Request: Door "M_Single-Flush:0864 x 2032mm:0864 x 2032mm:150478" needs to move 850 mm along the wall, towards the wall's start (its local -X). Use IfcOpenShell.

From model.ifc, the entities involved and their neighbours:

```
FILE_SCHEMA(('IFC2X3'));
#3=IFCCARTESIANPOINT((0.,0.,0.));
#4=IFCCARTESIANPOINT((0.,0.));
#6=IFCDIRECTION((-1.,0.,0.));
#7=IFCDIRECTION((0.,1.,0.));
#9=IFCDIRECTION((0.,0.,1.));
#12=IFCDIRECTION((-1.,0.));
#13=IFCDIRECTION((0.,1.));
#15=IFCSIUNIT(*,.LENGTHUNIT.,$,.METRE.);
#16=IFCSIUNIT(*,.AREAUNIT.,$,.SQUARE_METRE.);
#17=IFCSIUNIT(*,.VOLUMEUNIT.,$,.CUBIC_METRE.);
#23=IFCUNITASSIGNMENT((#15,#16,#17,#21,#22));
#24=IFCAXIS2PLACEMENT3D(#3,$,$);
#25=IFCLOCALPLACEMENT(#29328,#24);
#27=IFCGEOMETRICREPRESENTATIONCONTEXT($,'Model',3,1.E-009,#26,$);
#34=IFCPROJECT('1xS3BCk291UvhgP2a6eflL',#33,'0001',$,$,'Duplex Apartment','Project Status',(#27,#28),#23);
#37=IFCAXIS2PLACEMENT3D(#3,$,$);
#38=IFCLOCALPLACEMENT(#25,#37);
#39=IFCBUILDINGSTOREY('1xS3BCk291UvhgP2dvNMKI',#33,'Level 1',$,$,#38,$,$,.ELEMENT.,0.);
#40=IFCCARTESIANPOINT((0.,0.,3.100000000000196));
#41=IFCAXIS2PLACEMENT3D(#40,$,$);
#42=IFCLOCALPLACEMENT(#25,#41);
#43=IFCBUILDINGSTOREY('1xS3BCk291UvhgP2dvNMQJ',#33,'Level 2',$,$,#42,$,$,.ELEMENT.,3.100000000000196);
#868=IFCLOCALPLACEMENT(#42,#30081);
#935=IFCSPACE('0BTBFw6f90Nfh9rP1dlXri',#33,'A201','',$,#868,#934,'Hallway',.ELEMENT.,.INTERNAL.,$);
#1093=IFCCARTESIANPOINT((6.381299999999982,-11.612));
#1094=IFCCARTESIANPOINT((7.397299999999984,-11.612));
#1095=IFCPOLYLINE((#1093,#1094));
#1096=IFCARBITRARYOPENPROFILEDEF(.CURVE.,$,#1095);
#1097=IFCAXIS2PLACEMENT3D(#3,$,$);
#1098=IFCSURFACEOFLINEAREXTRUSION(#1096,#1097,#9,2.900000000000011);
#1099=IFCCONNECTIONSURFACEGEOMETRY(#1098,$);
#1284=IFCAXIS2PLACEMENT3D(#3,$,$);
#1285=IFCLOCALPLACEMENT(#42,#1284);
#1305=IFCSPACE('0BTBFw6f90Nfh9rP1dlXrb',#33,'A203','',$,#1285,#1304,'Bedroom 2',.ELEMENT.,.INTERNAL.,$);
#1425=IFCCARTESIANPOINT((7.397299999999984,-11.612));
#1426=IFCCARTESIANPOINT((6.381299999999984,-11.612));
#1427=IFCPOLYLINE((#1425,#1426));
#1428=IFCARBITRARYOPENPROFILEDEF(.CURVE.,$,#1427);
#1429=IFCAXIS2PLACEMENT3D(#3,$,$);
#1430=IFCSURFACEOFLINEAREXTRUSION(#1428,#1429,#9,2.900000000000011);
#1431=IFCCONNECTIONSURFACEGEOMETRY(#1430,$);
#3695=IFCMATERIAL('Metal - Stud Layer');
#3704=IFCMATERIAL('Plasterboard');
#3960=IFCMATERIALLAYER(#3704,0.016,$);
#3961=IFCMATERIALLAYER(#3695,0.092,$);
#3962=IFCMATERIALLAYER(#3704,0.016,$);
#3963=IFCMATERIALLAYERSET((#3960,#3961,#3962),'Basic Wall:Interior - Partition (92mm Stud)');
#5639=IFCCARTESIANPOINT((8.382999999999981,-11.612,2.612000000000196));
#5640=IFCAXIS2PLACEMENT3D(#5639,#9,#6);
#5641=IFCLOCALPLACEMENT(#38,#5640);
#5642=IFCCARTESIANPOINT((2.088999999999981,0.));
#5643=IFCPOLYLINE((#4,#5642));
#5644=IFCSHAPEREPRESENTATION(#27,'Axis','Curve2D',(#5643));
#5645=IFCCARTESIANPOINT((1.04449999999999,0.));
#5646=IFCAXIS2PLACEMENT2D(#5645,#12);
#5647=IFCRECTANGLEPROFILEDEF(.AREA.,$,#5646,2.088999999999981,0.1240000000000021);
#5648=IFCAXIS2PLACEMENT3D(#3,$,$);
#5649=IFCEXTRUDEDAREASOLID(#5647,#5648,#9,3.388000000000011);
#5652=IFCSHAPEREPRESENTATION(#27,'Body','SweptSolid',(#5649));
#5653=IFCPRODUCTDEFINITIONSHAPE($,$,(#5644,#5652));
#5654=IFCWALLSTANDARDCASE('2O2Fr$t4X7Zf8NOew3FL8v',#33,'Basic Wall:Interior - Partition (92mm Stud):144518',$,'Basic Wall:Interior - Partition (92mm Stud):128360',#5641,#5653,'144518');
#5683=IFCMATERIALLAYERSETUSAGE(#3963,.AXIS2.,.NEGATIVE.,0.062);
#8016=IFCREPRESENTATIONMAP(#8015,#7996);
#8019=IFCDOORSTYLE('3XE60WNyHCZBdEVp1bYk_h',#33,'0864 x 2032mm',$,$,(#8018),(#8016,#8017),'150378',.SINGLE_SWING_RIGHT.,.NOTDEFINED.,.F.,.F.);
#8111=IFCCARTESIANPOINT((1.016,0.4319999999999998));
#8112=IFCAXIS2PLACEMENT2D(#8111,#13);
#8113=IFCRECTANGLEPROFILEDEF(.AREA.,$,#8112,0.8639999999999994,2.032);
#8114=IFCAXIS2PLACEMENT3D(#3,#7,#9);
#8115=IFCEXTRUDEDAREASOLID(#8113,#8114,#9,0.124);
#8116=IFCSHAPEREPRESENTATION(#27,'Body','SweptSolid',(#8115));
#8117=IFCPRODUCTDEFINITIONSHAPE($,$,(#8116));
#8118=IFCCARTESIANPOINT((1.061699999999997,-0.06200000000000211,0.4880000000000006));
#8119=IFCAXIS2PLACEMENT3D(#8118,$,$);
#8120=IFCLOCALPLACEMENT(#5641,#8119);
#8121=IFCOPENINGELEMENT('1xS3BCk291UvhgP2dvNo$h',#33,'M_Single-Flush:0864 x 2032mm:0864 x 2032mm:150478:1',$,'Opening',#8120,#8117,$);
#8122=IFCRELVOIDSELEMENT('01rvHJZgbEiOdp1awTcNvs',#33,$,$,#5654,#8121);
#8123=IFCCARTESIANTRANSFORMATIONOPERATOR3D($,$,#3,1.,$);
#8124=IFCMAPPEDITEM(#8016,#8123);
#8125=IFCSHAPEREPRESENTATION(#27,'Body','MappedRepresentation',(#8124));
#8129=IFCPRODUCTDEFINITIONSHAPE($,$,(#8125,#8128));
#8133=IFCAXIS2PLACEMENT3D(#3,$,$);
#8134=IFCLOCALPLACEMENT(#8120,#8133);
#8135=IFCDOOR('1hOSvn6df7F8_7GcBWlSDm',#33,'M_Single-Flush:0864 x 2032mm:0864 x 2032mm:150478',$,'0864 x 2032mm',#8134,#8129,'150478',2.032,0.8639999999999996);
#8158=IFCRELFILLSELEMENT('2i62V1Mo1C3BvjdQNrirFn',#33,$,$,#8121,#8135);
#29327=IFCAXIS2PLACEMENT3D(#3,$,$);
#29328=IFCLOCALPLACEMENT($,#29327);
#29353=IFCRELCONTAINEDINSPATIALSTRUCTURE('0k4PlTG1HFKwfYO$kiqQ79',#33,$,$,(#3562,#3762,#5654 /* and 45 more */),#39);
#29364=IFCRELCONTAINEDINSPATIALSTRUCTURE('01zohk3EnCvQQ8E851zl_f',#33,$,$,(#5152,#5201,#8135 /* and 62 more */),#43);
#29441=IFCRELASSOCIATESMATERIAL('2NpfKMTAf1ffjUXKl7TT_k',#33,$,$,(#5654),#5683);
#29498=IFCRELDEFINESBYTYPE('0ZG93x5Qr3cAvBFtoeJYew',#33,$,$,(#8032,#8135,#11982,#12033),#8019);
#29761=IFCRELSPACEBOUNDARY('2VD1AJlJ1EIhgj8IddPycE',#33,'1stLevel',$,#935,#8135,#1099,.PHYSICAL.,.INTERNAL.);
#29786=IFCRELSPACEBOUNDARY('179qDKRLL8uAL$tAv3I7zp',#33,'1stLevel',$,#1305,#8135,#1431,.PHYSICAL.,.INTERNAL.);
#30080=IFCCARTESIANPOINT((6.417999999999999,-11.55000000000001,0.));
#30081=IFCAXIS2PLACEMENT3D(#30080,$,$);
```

```python
import numpy as np
import ifcopenshell
import ifcopenshell.api.geometry
import ifcopenshell.util.placement
import ifcopenshell.util.unit

model = ifcopenshell.open("model.ifc")
unit_scale = ifcopenshell.util.unit.calculate_unit_scale(model)

door = model.by_guid("1hOSvn6df7F8_7GcBWlSDm")
opening = door.FillsVoids[0].RelatingOpeningElement
wall = opening.VoidsElements[0].RelatingBuildingElement

wall_matrix = ifcopenshell.util.placement.get_local_placement(wall.ObjectPlacement)
shift = wall_matrix[:3, 0] * -0.85 / unit_scale
before = ifcopenshell.util.placement.get_local_placement(door.ObjectPlacement)[:3, 3].copy()

# The door is placed relative to its opening, so it follows when the opening moves.
matrix = ifcopenshell.util.placement.get_local_placement(opening.ObjectPlacement)
matrix[:3, 3] += shift
ifcopenshell.api.geometry.edit_object_placement(
    model, product=opening, matrix=matrix, is_si=False, should_transform_children=True
)

# Space boundary surfaces are stored in each space's coordinates; move them too.
for rel in door.ProvidesBoundaries:
    if not rel.ConnectionGeometry:
        continue
    surface = rel.ConnectionGeometry.SurfaceOnRelatingElement
    space_matrix = ifcopenshell.util.placement.get_local_placement(rel.RelatingSpace.ObjectPlacement)
    point = np.array(surface.Position.Location.Coordinates) + space_matrix[:3, :3].T @ shift
    surface.Position = model.createIfcAxis2Placement3D(
        model.createIfcCartesianPoint(point.tolist()), surface.Position.Axis, surface.Position.RefDirection
    )

after = ifcopenshell.util.placement.get_local_placement(door.ObjectPlacement)[:3, 3]
print("door moved by", (after - before).round(3) + 0.0)

model.write("model_rev.ifc")
```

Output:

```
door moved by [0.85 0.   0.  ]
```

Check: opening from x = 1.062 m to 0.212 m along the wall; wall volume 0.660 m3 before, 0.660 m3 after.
